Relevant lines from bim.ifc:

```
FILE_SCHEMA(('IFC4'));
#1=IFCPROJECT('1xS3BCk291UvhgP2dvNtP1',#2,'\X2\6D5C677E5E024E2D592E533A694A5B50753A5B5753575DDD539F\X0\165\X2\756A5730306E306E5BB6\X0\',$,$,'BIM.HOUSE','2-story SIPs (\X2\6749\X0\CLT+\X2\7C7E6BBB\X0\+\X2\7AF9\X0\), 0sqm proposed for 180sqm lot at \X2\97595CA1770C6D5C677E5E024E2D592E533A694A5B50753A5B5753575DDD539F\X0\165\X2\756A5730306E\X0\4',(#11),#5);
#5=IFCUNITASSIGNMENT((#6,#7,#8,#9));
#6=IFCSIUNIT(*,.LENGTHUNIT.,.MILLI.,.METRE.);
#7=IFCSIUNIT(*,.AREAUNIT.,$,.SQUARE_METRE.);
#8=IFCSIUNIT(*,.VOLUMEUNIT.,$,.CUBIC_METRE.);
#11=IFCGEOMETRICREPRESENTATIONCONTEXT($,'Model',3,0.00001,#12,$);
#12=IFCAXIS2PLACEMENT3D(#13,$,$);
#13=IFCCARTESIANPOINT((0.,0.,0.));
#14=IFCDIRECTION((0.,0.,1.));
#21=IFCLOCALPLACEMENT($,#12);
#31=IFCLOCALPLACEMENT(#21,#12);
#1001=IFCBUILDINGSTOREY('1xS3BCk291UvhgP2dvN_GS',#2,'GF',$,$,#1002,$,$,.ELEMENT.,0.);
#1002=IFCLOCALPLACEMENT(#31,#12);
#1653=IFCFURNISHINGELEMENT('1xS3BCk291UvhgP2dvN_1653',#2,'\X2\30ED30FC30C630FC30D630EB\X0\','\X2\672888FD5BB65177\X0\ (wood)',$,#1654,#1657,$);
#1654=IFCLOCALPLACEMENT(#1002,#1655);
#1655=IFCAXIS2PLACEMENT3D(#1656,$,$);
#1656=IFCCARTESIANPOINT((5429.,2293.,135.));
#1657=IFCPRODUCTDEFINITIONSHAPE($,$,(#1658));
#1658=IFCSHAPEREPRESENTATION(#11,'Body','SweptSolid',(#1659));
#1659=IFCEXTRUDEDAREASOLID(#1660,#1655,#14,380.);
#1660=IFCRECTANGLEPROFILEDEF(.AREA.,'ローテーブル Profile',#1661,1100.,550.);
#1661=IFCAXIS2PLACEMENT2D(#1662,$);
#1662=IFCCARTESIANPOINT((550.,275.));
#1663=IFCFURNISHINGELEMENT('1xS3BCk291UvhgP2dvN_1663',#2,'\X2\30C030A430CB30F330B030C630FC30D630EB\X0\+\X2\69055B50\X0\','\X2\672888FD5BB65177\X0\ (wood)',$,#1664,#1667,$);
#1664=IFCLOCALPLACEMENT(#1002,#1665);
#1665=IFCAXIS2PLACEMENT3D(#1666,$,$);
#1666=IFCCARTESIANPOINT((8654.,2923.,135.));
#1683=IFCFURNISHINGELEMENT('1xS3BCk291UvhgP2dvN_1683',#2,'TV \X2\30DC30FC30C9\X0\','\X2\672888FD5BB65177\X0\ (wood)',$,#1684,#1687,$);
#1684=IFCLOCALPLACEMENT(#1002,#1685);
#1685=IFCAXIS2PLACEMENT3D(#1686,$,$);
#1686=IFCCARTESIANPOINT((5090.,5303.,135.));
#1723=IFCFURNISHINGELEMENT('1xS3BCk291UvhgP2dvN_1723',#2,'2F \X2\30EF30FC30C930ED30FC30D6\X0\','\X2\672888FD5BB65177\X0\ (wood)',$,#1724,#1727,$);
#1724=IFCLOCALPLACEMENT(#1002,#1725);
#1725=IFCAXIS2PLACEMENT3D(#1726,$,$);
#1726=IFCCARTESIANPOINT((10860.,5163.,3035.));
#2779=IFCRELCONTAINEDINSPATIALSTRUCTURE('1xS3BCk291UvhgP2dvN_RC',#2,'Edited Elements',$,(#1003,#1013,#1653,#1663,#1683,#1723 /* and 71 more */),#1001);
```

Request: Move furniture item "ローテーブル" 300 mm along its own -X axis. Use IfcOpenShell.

```python
import ifcopenshell
import ifcopenshell.api.geometry
import ifcopenshell.util.placement
import ifcopenshell.util.unit

model = ifcopenshell.open("bim.ifc")
unit_scale = ifcopenshell.util.unit.calculate_unit_scale(model)

item = model.by_id(1653)
matrix = ifcopenshell.util.placement.get_local_placement(item.ObjectPlacement)
matrix[:3, 3] -= matrix[:3, 0] * 0.3 / unit_scale
ifcopenshell.api.geometry.edit_object_placement(model, product=item, matrix=matrix, is_si=False)

print(ifcopenshell.util.placement.get_local_placement(item.ObjectPlacement).round(3) + 0.0)

model.write("bim_v2.ifc")
```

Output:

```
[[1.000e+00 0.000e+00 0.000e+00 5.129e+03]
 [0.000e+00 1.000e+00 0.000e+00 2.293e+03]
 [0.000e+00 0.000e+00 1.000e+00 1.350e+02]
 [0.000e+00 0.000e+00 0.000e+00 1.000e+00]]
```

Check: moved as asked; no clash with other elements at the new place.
